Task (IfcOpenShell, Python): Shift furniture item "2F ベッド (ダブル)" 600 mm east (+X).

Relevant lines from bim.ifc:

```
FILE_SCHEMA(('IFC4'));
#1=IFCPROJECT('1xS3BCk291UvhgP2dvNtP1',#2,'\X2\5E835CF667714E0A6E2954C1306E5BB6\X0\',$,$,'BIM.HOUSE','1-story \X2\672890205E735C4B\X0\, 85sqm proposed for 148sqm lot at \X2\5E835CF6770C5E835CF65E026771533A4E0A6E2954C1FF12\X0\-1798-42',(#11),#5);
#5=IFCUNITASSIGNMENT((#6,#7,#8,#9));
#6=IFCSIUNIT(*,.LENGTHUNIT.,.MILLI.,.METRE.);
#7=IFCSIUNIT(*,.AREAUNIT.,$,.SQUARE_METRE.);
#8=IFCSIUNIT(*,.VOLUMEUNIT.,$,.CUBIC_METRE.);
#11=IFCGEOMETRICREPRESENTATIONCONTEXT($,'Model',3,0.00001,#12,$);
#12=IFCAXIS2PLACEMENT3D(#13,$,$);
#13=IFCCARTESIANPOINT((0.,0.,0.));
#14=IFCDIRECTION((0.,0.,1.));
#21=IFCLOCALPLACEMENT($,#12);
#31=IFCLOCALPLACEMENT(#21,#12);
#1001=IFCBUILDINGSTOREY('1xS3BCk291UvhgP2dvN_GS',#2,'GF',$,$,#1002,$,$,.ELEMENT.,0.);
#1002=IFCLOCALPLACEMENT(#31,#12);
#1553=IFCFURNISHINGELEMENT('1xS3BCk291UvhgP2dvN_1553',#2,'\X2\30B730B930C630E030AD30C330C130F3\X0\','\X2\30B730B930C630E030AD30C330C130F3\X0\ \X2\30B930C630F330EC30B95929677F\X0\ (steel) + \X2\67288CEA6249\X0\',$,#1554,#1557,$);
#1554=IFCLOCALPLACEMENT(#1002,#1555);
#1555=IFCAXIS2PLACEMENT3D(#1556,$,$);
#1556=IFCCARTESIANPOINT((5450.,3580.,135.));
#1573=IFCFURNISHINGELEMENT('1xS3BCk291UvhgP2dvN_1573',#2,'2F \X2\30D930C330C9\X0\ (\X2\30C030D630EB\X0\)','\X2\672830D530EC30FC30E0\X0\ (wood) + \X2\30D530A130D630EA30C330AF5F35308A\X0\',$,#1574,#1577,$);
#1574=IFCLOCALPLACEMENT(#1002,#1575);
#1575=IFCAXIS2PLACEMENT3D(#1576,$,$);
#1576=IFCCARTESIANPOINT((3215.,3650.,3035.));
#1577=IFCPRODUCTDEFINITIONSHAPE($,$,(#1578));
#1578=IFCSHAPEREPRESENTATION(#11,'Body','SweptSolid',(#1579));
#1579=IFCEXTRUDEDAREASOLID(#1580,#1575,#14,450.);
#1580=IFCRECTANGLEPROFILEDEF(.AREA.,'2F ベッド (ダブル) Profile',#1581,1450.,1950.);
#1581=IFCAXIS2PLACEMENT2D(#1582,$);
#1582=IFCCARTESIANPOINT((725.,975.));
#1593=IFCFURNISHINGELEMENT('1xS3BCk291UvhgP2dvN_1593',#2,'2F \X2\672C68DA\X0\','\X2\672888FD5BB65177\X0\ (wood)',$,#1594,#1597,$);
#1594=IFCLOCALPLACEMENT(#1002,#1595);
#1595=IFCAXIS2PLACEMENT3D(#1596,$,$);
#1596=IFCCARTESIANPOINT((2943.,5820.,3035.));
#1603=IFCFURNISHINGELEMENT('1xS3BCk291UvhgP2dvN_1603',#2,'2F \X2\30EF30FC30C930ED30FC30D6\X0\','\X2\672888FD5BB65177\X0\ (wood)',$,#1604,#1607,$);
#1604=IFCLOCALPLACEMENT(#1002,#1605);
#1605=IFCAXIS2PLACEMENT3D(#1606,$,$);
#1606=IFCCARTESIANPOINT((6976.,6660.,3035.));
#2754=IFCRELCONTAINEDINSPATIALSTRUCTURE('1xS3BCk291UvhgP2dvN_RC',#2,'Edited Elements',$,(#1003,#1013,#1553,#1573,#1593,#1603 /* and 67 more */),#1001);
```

```python
import ifcopenshell
import ifcopenshell.api.geometry
import ifcopenshell.util.placement
import ifcopenshell.util.unit

model = ifcopenshell.open("bim.ifc")
unit_scale = ifcopenshell.util.unit.calculate_unit_scale(model)

item = model.by_guid("1xS3BCk291UvhgP2dvN_1573")
matrix = ifcopenshell.util.placement.get_local_placement(item.ObjectPlacement)
matrix[0, 3] += 0.6 / unit_scale
ifcopenshell.api.geometry.edit_object_placement(model, product=item, matrix=matrix, is_si=False)

print(ifcopenshell.util.placement.get_local_placement(item.ObjectPlacement).round(3) + 0.0)

model.write("bim_updated.ifc")
```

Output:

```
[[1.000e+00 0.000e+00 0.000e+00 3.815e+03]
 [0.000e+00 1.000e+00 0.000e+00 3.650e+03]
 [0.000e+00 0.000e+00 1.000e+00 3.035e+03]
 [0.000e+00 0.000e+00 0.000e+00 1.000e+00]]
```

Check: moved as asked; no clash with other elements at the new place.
